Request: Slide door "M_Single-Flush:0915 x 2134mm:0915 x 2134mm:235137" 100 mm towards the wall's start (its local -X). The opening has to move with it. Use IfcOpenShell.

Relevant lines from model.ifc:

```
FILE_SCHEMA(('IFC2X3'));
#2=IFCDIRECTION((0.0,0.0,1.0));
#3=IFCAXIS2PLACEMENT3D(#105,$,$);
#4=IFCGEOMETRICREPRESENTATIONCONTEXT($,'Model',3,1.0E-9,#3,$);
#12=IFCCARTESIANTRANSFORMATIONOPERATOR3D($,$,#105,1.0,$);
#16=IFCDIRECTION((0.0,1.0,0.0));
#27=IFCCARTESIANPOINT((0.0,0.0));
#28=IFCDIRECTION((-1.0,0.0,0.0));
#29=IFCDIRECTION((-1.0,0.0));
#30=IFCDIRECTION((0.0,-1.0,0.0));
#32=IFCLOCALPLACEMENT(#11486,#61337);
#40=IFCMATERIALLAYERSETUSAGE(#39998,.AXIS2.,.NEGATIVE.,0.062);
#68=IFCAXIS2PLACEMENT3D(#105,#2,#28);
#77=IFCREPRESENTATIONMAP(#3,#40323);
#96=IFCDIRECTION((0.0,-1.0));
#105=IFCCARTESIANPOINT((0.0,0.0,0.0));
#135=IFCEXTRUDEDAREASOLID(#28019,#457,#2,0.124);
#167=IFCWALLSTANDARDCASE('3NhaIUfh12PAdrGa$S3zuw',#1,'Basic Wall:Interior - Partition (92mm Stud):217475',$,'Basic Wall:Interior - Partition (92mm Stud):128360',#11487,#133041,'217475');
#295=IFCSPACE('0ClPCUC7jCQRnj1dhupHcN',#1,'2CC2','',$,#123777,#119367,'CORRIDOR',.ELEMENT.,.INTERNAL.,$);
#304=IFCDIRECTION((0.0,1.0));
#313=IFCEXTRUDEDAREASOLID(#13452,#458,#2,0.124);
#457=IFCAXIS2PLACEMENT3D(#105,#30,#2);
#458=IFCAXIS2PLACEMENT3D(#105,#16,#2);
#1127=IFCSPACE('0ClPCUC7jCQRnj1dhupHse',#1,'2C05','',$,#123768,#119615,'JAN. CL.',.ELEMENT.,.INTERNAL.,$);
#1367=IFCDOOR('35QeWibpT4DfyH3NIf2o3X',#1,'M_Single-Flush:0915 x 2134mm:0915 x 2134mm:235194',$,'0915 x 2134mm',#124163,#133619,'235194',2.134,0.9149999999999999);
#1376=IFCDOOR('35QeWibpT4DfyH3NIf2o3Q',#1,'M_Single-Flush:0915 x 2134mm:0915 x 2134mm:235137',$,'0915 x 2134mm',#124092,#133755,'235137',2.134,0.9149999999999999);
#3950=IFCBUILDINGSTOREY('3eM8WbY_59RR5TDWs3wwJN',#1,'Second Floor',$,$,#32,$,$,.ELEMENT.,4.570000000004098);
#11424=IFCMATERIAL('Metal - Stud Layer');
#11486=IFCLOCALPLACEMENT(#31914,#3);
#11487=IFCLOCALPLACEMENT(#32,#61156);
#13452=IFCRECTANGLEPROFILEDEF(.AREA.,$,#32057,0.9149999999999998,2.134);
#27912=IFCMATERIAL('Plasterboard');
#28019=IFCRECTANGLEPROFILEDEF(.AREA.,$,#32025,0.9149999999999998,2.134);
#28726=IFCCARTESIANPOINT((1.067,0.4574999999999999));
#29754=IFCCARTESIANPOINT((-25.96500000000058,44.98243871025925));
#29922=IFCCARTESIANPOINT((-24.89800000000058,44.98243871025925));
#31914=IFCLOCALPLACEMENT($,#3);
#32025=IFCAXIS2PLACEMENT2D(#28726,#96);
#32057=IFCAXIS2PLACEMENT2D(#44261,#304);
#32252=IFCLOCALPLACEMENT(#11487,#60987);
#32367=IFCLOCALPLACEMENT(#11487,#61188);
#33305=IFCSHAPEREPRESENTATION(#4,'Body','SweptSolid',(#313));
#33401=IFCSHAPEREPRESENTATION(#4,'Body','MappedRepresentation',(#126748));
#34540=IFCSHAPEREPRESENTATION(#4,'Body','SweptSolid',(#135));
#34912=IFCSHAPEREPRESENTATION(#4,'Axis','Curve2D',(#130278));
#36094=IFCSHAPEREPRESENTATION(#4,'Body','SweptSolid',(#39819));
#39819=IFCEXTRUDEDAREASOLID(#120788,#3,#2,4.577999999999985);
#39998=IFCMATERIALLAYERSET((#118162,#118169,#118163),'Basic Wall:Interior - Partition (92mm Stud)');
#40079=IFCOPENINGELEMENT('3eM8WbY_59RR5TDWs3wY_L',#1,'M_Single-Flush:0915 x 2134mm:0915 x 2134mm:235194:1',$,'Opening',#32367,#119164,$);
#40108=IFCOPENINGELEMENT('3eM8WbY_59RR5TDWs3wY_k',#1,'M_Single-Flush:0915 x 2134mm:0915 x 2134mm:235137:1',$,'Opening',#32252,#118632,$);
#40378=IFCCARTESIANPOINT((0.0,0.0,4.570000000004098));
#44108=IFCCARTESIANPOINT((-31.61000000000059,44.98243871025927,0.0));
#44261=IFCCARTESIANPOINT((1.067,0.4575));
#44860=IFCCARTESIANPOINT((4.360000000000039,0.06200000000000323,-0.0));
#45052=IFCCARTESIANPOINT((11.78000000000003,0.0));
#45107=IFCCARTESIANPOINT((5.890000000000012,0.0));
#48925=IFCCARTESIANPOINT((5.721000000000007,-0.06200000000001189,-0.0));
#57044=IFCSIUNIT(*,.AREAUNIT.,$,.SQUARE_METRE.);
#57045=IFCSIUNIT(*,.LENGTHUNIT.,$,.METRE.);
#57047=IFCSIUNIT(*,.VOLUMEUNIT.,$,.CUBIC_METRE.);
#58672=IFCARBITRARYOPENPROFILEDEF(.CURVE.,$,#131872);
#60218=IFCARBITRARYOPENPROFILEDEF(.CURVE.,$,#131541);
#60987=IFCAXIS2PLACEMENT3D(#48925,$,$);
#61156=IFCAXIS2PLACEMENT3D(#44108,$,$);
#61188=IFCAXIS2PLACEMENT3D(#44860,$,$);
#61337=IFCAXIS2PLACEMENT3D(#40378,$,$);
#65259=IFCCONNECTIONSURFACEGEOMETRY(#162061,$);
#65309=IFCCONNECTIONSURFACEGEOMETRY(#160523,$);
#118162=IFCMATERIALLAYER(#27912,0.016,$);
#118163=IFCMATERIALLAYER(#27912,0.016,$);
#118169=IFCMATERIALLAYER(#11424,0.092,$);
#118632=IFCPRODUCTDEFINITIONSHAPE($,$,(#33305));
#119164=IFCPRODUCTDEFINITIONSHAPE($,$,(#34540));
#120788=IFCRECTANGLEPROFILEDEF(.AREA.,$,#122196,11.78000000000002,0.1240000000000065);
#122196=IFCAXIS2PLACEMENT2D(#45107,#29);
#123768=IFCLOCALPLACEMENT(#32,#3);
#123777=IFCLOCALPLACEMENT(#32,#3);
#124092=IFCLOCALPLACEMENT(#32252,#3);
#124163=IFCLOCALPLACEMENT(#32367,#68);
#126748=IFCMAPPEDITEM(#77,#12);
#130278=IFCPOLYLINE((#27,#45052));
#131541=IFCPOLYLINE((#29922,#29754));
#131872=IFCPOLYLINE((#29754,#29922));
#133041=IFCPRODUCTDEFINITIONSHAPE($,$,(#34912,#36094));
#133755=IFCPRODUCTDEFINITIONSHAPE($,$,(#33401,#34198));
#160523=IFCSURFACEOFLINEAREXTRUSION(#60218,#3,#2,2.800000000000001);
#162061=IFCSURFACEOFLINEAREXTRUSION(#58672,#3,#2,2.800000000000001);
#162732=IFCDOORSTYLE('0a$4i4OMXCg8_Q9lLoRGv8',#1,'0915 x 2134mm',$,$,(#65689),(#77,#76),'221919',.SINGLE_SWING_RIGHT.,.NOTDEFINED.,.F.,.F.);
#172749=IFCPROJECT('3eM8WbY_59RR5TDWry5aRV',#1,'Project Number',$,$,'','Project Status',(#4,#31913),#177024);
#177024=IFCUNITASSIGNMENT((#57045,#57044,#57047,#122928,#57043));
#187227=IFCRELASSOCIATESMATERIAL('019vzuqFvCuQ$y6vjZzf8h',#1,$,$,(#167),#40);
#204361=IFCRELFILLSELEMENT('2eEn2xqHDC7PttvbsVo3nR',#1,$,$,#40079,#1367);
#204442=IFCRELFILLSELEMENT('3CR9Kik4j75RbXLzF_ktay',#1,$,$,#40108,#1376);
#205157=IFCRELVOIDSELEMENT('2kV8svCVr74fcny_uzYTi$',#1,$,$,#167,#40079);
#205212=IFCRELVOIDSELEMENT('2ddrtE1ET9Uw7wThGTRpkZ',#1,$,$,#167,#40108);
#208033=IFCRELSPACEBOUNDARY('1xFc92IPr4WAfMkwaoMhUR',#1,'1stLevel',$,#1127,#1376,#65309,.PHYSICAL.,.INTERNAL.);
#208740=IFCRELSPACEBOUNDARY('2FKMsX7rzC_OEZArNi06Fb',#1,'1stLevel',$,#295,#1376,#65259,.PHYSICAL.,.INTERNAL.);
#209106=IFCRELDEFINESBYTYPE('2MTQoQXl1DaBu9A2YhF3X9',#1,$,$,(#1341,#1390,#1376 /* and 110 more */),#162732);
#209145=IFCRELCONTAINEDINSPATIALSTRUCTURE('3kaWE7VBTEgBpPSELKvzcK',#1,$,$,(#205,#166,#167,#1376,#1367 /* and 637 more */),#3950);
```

```python
import numpy as np
import ifcopenshell
import ifcopenshell.api.geometry
import ifcopenshell.util.placement

model = ifcopenshell.open("model.ifc")

door = model.by_guid("35QeWibpT4DfyH3NIf2o3Q")
opening = door.FillsVoids[0].RelatingOpeningElement
wall = opening.VoidsElements[0].RelatingBuildingElement

wall_matrix = ifcopenshell.util.placement.get_local_placement(wall.ObjectPlacement)
shift = wall_matrix[:3, 0] * -0.1
before = ifcopenshell.util.placement.get_local_placement(door.ObjectPlacement)[:3, 3].copy()

# The door is placed relative to its opening, so it follows when the opening moves.
matrix = ifcopenshell.util.placement.get_local_placement(opening.ObjectPlacement)
matrix[:3, 3] += shift
ifcopenshell.api.geometry.edit_object_placement(
    model, product=opening, matrix=matrix, is_si=False, should_transform_children=True
)

# Space boundary surfaces are stored in each space's coordinates; move them too.
for rel in door.ProvidesBoundaries:
    if not rel.ConnectionGeometry:
        continue
    surface = rel.ConnectionGeometry.SurfaceOnRelatingElement
    space_matrix = ifcopenshell.util.placement.get_local_placement(rel.RelatingSpace.ObjectPlacement)
    point = np.array(surface.Position.Location.Coordinates) + space_matrix[:3, :3].T @ shift
    surface.Position = model.createIfcAxis2Placement3D(
        model.createIfcCartesianPoint(point.tolist()), surface.Position.Axis, surface.Position.RefDirection
    )

after = ifcopenshell.util.placement.get_local_placement(door.ObjectPlacement)[:3, 3]
print("door moved by", (after - before).round(3) + 0.0)

model.write("model_updated.ifc")
```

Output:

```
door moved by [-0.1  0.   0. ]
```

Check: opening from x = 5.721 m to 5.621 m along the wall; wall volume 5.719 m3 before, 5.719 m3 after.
